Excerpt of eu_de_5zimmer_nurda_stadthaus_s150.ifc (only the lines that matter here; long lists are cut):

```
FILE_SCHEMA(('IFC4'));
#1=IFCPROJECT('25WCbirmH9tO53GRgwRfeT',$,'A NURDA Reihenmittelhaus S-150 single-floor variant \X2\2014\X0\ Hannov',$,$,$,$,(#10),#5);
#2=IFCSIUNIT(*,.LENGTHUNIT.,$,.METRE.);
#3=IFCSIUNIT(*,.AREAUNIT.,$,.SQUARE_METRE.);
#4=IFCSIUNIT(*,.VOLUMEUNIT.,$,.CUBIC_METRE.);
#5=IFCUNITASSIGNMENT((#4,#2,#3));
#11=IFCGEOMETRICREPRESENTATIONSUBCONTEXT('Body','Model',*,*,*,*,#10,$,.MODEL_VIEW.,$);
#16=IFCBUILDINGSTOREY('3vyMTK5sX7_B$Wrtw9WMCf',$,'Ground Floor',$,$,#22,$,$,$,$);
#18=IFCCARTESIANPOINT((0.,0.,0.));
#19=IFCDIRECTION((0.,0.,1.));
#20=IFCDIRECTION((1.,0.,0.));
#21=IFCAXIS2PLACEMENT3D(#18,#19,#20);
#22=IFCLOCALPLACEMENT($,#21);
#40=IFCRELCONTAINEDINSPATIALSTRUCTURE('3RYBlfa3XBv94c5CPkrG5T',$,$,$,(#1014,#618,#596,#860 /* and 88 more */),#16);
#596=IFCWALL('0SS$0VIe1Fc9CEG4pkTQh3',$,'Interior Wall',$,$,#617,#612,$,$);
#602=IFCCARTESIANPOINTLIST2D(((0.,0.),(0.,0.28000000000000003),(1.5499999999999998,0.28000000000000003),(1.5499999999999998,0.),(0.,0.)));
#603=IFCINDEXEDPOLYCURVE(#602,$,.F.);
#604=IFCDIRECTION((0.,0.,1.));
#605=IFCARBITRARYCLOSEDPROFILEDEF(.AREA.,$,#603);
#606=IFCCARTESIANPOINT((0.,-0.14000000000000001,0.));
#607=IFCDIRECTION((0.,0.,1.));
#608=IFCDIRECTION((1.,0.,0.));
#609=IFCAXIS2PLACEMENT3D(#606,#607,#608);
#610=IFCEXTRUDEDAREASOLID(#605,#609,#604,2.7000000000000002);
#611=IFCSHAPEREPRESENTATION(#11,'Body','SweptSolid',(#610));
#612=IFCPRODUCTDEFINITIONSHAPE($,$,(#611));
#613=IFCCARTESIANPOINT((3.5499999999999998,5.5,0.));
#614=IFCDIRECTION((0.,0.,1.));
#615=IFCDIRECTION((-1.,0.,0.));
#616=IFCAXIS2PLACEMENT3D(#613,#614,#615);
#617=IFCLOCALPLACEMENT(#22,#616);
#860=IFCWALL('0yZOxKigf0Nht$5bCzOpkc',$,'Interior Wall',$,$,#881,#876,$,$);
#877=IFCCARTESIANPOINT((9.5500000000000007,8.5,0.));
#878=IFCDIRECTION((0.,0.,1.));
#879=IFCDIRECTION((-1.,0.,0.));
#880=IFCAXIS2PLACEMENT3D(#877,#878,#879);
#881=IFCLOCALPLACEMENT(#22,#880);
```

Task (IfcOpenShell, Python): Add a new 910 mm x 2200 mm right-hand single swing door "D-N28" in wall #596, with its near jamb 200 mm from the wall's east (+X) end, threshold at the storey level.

```python
import numpy as np
import ifcopenshell
import ifcopenshell.api.feature
import ifcopenshell.api.geometry
import ifcopenshell.api.root
import ifcopenshell.api.spatial
import ifcopenshell.geom
import ifcopenshell.util.element
import ifcopenshell.util.placement
import ifcopenshell.util.representation
import ifcopenshell.util.shape
import ifcopenshell.util.unit

model = ifcopenshell.open("eu_de_5zimmer_nurda_stadthaus_s150.ifc")
unit_scale = ifcopenshell.util.unit.calculate_unit_scale(model)
settings = ifcopenshell.geom.settings()


def volume(element):
    """Net volume in cubic metres, openings subtracted."""
    shape = ifcopenshell.geom.create_shape(settings, element)
    return ifcopenshell.util.shape.get_volume(shape.geometry)


wall = model.by_guid("0SS$0VIe1Fc9CEG4pkTQh3")
storey = ifcopenshell.util.element.get_container(wall, ifc_class="IfcBuildingStorey")
context = ifcopenshell.util.representation.get_context(model, "Model", "Body", "MODEL_VIEW")
before = volume(wall)

width, height, from_end, sill = 0.91, 2.2, 0.2, 0.0  # metres

# The wall runs along its own X axis, and the end named is its -X end.
wall_shape = ifcopenshell.geom.create_shape(settings, wall)
x, y, z = ifcopenshell.util.shape.get_vertices(wall_shape.geometry).T
start = x.min() + from_end
face, thickness = float(y.min()), float(y.max() - y.min())
wall_matrix = ifcopenshell.util.placement.get_local_placement(wall.ObjectPlacement)
level = ifcopenshell.util.placement.get_local_placement(storey.ObjectPlacement)[2, 3]


def in_wall(x, y):
    """Placement at x, y metres in the wall's axes, at sill height."""
    matrix = wall_matrix.copy()
    matrix[:, 3] = wall_matrix @ np.array([x / unit_scale, y / unit_scale, 0.0, 1.0])
    matrix[2, 3] = level + sill / unit_scale
    return matrix


# Opening: a box that overshoots both wall faces by 50 mm.
opening = ifcopenshell.api.root.create_entity(model, ifc_class="IfcOpeningElement", predefined_type="OPENING")
box = ifcopenshell.api.geometry.add_wall_representation(
    model, context=context, length=width, height=height, thickness=thickness + 0.1
)
ifcopenshell.api.geometry.assign_representation(model, product=opening, representation=box)
ifcopenshell.api.geometry.edit_object_placement(model, product=opening, matrix=in_wall(start, face - 0.05), is_si=False)
ifcopenshell.api.feature.add_feature(model, feature=opening, element=wall)

door = ifcopenshell.api.root.create_entity(model, ifc_class="IfcDoor", name="D-N28", predefined_type="DOOR")
door.OverallWidth, door.OverallHeight = width / unit_scale, height / unit_scale
door.OperationType = "SINGLE_SWING_RIGHT"
body = ifcopenshell.api.geometry.add_door_representation(
    model,
    context=context,
    overall_width=door.OverallWidth,
    overall_height=door.OverallHeight,
    operation_type="SINGLE_SWING_RIGHT",
    lining_properties={"LiningDepth": thickness / unit_scale, "ThresholdDepth": thickness / unit_scale},
)
ifcopenshell.api.geometry.assign_representation(model, product=door, representation=body)
ifcopenshell.api.spatial.assign_container(model, products=[door], relating_structure=storey)
ifcopenshell.api.feature.add_filling(model, opening=opening, element=door)

# The lining spans the wall, so the door starts at the wall face.
ifcopenshell.api.geometry.edit_object_placement(model, product=door, matrix=in_wall(start, face), is_si=False)

after = volume(wall)

print(f"wall volume {before:.3f} -> {after:.3f} m3")

model.write("eu_de_5zimmer_nurda_stadthaus_s150_edited.ifc")
```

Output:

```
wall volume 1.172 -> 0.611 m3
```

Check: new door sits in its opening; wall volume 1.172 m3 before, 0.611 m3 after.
